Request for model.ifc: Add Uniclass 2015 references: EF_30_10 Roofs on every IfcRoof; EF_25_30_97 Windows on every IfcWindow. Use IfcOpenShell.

First a look at what the model holds.

```python
import ifcopenshell

model = ifcopenshell.open("model.ifc")
print(model.schema)
print("classifications:", [c.Name for c in model.by_type("IfcClassification")])
for ifc_class in ("IfcDoor", "IfcRoof", "IfcStair", "IfcWall", "IfcWindow"):
    print(ifc_class, len(model.by_type(ifc_class)))
```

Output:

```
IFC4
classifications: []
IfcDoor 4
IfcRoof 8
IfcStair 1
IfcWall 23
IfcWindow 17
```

```python
import ifcopenshell
import ifcopenshell.api.classification

model = ifcopenshell.open("model.ifc")

system = ifcopenshell.api.classification.add_classification(model, classification="Uniclass 2015")

codes = {
    "IfcRoof": ("EF_30_10", "Roofs"),
    "IfcWindow": ("EF_25_30_97", "Windows"),
}
for ifc_class, (code, name) in codes.items():
    products = model.by_type(ifc_class)
    ifcopenshell.api.classification.add_reference(
        model, products=products, classification=system, identification=code, name=name
    )
    print(code, len(products))

model.write("model_edited.ifc")
```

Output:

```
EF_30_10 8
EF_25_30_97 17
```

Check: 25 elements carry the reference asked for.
